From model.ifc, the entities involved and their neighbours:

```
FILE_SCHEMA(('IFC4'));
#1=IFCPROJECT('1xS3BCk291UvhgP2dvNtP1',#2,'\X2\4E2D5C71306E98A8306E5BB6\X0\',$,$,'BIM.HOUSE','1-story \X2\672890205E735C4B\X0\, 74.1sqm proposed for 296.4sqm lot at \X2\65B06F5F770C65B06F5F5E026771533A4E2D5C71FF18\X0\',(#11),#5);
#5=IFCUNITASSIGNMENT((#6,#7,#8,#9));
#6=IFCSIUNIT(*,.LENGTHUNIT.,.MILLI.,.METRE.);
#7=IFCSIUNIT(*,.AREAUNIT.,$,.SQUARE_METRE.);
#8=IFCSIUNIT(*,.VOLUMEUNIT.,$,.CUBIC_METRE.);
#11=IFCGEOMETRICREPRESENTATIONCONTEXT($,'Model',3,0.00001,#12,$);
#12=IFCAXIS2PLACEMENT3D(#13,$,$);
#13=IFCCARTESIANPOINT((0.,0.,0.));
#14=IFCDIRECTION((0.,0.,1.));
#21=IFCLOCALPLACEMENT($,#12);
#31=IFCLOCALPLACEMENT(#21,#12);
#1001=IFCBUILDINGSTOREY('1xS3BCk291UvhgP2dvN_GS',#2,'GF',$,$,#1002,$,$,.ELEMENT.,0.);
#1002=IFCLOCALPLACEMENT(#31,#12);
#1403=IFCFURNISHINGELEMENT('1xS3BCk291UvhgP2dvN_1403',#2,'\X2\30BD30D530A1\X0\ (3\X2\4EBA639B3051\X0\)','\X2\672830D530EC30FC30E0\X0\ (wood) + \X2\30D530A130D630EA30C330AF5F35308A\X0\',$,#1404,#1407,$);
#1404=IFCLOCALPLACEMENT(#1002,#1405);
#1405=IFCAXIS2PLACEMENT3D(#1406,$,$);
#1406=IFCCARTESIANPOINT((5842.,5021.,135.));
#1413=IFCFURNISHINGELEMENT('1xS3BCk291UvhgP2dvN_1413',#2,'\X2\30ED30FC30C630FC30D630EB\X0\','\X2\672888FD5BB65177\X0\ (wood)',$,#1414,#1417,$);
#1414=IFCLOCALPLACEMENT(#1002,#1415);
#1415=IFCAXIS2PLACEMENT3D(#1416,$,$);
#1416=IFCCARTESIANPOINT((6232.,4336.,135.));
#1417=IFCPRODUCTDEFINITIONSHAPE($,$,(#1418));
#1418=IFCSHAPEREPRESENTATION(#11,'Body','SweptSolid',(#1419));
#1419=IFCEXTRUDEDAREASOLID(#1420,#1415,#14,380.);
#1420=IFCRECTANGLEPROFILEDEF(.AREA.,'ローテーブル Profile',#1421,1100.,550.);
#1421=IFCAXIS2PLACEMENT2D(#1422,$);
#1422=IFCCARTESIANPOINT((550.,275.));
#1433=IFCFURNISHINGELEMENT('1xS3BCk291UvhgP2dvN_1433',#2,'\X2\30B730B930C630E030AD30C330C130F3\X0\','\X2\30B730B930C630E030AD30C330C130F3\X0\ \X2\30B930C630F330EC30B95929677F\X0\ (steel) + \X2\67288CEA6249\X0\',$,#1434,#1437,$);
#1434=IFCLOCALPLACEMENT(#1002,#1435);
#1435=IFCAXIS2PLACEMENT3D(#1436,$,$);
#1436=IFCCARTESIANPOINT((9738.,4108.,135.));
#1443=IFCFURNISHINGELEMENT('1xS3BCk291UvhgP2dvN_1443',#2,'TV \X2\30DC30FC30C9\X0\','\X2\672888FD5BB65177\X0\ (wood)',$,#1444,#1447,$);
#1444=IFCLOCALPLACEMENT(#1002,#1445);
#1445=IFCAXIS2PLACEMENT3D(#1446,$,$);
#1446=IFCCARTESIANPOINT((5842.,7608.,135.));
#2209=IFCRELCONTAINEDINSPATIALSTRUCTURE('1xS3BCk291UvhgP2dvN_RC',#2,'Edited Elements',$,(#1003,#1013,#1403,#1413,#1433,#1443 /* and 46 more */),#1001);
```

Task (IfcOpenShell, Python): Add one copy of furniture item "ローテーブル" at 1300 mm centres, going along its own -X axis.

```python
import ifcopenshell
import ifcopenshell.api.geometry
import ifcopenshell.api.root
import ifcopenshell.util.element
import ifcopenshell.util.placement

model = ifcopenshell.open("model.ifc")


def reuse_history(source, copy):
    """copy_class also copies each property set's owner history, people and application; keep the originals."""
    for rel in copy.IsDefinedBy:
        if rel.is_a("IfcRelDefinesByProperties") and (history := rel.RelatingPropertyDefinition.OwnerHistory):
            rel.RelatingPropertyDefinition.OwnerHistory = source.OwnerHistory
            ifcopenshell.util.element.remove_deep2(model, history)


source = model.by_guid("1xS3BCk291UvhgP2dvN_1413")
base = ifcopenshell.util.placement.get_local_placement(source.ObjectPlacement)
step = -base[:3, 0] * 1300.0

for i in range(1, 2):
    copy = ifcopenshell.api.root.copy_class(model, product=source)
    copy.Representation = ifcopenshell.util.element.copy_deep(
        model, source.Representation, exclude=["IfcGeometricRepresentationContext", "IfcRepresentationMap"]
    )
    reuse_history(source, copy)
    matrix = base.copy()
    matrix[:3, 3] += i * step
    print("added at", matrix[:3, 3].round(3) + 0.0)
    ifcopenshell.api.geometry.edit_object_placement(model, product=copy, matrix=matrix, is_si=False)

model.write("model_updated.ifc")
```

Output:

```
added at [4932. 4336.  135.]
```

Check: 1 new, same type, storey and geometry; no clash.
